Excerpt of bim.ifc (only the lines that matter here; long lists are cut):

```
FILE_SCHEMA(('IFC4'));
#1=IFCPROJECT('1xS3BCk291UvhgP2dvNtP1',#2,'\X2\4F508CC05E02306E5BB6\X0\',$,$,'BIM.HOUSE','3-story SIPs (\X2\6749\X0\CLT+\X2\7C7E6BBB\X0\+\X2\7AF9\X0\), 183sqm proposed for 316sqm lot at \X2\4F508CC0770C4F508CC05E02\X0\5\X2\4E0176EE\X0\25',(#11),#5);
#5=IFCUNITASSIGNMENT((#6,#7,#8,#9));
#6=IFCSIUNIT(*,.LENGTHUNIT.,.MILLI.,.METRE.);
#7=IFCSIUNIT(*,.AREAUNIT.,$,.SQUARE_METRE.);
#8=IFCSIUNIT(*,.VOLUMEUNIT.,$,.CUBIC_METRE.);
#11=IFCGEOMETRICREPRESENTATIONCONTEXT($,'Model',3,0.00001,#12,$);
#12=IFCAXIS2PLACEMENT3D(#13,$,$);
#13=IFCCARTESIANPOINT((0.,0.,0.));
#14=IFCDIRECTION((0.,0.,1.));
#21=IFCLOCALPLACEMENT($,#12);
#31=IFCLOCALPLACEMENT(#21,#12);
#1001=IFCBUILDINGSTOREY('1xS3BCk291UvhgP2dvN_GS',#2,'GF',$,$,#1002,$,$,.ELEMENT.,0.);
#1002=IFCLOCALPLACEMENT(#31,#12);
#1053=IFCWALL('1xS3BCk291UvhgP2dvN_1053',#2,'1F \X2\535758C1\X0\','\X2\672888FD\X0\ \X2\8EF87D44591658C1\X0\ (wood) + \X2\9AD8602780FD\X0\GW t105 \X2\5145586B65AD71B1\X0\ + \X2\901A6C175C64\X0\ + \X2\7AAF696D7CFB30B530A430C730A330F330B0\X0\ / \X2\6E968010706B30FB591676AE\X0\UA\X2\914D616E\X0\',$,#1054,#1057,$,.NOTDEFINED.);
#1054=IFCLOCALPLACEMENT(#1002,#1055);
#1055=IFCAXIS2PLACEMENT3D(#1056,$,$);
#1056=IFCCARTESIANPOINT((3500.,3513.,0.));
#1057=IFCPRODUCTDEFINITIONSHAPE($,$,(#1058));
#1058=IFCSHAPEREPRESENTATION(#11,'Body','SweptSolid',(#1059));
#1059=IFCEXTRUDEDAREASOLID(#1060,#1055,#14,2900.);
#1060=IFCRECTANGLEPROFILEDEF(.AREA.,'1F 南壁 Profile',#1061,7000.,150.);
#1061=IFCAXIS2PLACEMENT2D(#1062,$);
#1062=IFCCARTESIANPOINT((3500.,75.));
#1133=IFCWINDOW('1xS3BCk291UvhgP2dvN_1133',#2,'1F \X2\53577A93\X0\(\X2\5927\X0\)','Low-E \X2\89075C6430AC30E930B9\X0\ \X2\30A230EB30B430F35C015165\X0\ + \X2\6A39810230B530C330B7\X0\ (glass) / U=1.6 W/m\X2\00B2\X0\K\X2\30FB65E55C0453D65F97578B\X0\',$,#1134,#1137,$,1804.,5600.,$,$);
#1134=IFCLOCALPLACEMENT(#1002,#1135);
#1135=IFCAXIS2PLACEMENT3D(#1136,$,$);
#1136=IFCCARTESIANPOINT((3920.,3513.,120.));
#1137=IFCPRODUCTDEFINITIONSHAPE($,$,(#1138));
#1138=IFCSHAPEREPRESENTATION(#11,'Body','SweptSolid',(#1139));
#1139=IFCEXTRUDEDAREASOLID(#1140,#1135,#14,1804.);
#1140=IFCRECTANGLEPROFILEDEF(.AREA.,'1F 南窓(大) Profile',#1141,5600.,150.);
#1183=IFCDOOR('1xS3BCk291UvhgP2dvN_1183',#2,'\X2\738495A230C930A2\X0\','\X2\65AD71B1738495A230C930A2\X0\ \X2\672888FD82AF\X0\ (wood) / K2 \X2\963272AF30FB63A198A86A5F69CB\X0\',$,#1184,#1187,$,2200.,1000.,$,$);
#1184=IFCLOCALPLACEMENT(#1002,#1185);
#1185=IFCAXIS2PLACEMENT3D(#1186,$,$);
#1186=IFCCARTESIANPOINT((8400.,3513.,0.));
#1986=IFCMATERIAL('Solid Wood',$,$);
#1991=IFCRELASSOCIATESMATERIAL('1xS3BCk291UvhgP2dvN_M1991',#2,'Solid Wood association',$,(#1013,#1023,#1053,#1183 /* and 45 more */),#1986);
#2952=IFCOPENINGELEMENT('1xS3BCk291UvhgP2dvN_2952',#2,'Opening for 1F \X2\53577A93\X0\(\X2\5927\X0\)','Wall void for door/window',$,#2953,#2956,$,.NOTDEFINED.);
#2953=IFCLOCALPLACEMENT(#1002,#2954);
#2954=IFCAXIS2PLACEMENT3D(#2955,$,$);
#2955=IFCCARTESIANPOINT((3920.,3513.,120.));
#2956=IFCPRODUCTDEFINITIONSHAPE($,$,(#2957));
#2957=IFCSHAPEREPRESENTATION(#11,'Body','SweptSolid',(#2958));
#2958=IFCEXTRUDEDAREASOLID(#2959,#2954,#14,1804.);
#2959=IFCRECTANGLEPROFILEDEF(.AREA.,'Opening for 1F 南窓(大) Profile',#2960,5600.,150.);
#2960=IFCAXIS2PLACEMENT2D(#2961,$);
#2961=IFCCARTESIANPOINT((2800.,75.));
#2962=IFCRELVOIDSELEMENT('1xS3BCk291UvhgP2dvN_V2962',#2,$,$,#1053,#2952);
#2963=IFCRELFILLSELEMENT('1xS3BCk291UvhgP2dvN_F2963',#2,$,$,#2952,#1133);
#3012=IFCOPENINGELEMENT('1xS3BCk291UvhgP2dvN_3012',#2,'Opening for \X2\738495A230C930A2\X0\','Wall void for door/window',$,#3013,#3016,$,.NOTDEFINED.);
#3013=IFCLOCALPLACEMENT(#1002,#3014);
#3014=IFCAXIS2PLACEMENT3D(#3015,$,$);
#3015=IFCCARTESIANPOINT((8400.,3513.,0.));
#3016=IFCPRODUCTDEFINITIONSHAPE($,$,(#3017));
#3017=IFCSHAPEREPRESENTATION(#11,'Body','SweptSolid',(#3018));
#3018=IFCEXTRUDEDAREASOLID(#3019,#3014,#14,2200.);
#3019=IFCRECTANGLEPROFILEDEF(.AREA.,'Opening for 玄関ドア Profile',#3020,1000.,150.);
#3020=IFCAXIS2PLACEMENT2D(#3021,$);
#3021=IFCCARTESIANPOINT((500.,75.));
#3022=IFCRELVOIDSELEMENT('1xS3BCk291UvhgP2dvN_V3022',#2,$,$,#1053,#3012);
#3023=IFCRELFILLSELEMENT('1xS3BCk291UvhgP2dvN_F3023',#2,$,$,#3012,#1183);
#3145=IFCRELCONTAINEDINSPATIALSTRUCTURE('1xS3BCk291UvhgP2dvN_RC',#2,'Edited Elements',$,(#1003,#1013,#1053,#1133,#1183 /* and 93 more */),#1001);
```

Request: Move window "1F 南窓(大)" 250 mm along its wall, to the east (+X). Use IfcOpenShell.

```python
import ifcopenshell
import ifcopenshell.api.geometry
import ifcopenshell.util.placement

model = ifcopenshell.open("bim.ifc")

window = model.by_id(1133)
opening = window.FillsVoids[0].RelatingOpeningElement
wall = opening.VoidsElements[0].RelatingBuildingElement

wall_matrix = ifcopenshell.util.placement.get_local_placement(wall.ObjectPlacement)
shift = wall_matrix[:3, 0] * 250.0
before = ifcopenshell.util.placement.get_local_placement(window.ObjectPlacement)[:3, 3].copy()

# The window is not placed relative to its opening, so move both.
for product in (opening, window):
    matrix = ifcopenshell.util.placement.get_local_placement(product.ObjectPlacement)
    matrix[:3, 3] += shift
    ifcopenshell.api.geometry.edit_object_placement(model, product=product, matrix=matrix, is_si=False)

after = ifcopenshell.util.placement.get_local_placement(window.ObjectPlacement)[:3, 3]
print("window moved by", (after - before).round(3) + 0.0)

model.write("bim_updated.ifc")
```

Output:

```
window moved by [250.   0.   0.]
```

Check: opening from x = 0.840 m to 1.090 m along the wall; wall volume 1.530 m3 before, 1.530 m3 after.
